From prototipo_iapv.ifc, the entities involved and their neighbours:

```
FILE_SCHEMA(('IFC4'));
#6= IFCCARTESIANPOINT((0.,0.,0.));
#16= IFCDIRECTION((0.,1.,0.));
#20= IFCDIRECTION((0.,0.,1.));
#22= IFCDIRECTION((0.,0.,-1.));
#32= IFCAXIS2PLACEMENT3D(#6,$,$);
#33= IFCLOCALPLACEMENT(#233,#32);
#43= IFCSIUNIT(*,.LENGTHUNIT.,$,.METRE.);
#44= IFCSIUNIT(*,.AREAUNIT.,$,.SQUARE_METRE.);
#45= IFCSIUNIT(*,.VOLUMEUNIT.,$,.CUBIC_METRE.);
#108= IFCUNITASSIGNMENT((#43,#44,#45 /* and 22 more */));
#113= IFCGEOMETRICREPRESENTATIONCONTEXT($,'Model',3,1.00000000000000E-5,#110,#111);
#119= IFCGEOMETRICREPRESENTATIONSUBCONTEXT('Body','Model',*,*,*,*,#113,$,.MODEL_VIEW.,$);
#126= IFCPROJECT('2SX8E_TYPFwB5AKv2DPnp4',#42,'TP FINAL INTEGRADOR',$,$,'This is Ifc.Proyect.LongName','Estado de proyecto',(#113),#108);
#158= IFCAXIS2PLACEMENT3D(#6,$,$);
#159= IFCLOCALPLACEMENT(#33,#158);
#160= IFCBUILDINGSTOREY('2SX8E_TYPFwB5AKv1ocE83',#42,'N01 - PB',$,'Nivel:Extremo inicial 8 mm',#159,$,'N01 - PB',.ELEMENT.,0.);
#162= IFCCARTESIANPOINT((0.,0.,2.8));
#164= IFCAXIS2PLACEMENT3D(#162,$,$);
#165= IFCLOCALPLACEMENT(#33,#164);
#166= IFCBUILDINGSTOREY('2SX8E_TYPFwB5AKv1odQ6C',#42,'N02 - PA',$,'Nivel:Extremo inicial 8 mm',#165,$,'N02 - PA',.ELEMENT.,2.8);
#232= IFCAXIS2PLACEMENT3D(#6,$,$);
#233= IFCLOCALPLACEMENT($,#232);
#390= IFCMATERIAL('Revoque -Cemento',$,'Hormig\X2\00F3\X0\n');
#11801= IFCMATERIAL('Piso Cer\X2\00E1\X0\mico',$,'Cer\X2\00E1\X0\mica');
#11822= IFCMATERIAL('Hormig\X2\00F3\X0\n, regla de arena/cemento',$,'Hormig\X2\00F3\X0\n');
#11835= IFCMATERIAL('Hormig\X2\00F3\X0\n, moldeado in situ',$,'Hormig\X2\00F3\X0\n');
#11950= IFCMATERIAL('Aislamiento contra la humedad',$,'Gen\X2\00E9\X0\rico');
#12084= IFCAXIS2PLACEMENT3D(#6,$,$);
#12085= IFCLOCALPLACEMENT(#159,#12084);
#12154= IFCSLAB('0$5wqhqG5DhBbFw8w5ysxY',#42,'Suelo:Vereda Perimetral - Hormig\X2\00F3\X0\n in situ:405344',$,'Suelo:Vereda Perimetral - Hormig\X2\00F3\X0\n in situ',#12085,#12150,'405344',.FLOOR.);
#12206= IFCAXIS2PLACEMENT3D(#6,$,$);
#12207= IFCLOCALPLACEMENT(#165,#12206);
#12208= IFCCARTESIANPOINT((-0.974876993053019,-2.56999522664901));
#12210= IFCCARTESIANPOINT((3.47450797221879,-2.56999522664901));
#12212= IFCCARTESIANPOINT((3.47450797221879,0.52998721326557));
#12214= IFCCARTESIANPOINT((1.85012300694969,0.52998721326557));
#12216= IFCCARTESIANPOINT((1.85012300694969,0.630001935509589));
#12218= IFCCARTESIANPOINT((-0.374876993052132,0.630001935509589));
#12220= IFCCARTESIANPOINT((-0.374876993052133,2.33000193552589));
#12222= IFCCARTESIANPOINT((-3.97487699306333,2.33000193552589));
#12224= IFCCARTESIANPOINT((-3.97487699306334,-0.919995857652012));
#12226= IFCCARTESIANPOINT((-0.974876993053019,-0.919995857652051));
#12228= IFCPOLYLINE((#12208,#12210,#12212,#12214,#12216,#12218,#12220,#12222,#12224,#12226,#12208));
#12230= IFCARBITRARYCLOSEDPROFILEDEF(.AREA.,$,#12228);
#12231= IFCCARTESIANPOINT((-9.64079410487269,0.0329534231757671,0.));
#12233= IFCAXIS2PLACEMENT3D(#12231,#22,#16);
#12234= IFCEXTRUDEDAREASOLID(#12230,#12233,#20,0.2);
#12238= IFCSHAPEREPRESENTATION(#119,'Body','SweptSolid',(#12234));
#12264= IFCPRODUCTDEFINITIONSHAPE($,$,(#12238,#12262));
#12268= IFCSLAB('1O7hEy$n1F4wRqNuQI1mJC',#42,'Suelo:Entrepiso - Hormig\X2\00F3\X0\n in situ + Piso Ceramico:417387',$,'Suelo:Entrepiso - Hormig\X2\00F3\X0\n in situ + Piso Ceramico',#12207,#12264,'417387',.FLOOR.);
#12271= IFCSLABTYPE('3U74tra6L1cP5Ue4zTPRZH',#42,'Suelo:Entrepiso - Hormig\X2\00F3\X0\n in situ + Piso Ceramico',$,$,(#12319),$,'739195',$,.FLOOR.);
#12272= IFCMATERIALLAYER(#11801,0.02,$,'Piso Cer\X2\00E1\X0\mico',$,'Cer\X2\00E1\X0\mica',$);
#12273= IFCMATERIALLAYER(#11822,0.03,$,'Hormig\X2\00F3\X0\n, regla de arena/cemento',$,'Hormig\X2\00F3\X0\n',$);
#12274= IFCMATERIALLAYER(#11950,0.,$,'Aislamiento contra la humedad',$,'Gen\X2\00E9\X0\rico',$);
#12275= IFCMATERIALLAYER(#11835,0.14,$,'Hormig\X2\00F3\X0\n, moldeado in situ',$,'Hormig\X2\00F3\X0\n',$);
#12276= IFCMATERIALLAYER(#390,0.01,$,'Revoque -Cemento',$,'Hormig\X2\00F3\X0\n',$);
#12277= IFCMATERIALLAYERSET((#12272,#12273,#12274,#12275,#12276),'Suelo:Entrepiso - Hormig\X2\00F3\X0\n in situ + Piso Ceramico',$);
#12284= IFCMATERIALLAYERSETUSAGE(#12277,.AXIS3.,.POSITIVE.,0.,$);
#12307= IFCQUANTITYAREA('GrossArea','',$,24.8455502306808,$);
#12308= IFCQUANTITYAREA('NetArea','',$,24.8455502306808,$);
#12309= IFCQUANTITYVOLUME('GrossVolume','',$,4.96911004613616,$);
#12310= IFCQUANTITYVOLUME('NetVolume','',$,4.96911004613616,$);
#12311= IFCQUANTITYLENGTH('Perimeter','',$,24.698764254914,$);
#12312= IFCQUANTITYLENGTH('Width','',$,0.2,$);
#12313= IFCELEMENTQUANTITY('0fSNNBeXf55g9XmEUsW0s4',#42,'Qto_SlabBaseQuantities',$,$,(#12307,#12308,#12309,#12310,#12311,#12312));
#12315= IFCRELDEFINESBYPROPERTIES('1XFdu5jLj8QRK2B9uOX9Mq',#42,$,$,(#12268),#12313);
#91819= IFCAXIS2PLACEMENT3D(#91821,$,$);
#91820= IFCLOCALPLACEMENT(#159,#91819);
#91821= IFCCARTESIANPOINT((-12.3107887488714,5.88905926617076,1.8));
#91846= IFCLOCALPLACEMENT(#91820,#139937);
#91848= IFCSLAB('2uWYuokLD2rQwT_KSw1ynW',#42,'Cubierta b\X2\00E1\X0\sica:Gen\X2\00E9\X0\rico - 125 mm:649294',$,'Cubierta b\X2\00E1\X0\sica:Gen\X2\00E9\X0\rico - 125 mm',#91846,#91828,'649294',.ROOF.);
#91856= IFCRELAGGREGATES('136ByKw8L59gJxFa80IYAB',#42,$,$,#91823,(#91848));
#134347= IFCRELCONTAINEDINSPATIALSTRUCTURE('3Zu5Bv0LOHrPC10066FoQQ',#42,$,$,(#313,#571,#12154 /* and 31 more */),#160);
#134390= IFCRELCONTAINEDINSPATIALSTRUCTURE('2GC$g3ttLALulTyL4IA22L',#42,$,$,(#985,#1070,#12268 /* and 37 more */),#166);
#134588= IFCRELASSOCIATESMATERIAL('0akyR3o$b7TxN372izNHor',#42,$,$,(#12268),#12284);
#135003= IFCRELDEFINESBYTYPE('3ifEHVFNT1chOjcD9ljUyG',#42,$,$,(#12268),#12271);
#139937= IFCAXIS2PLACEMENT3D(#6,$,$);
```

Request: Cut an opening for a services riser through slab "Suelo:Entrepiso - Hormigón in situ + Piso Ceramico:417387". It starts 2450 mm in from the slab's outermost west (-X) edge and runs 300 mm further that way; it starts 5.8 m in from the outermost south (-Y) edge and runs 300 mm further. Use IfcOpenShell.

```python
import numpy as np
import ifcopenshell
import ifcopenshell.api.feature
import ifcopenshell.api.geometry
import ifcopenshell.api.pset
import ifcopenshell.api.root
import ifcopenshell.geom
import ifcopenshell.util.element
import ifcopenshell.util.placement
import ifcopenshell.util.representation
import ifcopenshell.util.shape
import ifcopenshell.util.unit

model = ifcopenshell.open("prototipo_iapv.ifc")
unit_scale = ifcopenshell.util.unit.calculate_unit_scale(model)
area_scale = ifcopenshell.util.unit.calculate_unit_scale(model, "AREAUNIT")
volume_scale = ifcopenshell.util.unit.calculate_unit_scale(model, "VOLUMEUNIT")
settings = ifcopenshell.geom.settings()


def volume(element):
    """Net volume in cubic metres, openings subtracted."""
    shape = ifcopenshell.geom.create_shape(settings, element)
    return ifcopenshell.util.shape.get_volume(shape.geometry)


slab = model.by_guid("1O7hEy$n1F4wRqNuQI1mJC")
before = volume(slab)

# Extent in the slab's own axes, in metres. The edges named are its -X and -Y sides.
slab_shape = ifcopenshell.geom.create_shape(settings, slab)
vertices = ifcopenshell.util.shape.get_vertices(slab_shape.geometry)
x_min, y_min, bottom = vertices.min(axis=0)
top = vertices[:, 2].max()

opening = ifcopenshell.api.root.create_entity(model, ifc_class="IfcOpeningElement", name="Services riser opening", predefined_type="OPENING")
context = ifcopenshell.util.representation.get_context(model, "Model", "Body", "MODEL_VIEW")
width, depth = 0.3, 0.3
outline = [(0.0, 0.0), (width, 0.0), (width, depth), (0.0, depth), (0.0, 0.0)]
# Overshoot both faces by 50 mm so the cut is clean.
shape = ifcopenshell.api.geometry.add_slab_representation(
    model, context=context, depth=top - bottom + 0.1, polyline=outline
)
ifcopenshell.api.geometry.assign_representation(model, product=opening, representation=shape)

matrix = ifcopenshell.util.placement.get_local_placement(slab.ObjectPlacement)
matrix[:, 3] = matrix @ np.append(np.array([x_min + 2.45, y_min + 5.8, bottom - 0.05]) / unit_scale, 1.0)
ifcopenshell.api.geometry.edit_object_placement(model, product=opening, matrix=matrix, is_si=False)
ifcopenshell.api.feature.add_feature(model, feature=opening, element=slab)

after = volume(slab)

# Update the slab's stored quantities.
qto = model.by_id(ifcopenshell.util.element.get_pset(slab, "Qto_SlabBaseQuantities", should_inherit=False)["id"])
ifcopenshell.api.pset.edit_qto(model, qto=qto, properties={
    "NetArea": after / (top - bottom) / area_scale,
    "NetVolume": after / volume_scale,
})

print(f"slab volume {before:.3f} -> {after:.3f} m3")

model.write("prototipo_iapv_rev.ifc")
```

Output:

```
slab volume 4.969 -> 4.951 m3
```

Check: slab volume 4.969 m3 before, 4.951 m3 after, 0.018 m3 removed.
